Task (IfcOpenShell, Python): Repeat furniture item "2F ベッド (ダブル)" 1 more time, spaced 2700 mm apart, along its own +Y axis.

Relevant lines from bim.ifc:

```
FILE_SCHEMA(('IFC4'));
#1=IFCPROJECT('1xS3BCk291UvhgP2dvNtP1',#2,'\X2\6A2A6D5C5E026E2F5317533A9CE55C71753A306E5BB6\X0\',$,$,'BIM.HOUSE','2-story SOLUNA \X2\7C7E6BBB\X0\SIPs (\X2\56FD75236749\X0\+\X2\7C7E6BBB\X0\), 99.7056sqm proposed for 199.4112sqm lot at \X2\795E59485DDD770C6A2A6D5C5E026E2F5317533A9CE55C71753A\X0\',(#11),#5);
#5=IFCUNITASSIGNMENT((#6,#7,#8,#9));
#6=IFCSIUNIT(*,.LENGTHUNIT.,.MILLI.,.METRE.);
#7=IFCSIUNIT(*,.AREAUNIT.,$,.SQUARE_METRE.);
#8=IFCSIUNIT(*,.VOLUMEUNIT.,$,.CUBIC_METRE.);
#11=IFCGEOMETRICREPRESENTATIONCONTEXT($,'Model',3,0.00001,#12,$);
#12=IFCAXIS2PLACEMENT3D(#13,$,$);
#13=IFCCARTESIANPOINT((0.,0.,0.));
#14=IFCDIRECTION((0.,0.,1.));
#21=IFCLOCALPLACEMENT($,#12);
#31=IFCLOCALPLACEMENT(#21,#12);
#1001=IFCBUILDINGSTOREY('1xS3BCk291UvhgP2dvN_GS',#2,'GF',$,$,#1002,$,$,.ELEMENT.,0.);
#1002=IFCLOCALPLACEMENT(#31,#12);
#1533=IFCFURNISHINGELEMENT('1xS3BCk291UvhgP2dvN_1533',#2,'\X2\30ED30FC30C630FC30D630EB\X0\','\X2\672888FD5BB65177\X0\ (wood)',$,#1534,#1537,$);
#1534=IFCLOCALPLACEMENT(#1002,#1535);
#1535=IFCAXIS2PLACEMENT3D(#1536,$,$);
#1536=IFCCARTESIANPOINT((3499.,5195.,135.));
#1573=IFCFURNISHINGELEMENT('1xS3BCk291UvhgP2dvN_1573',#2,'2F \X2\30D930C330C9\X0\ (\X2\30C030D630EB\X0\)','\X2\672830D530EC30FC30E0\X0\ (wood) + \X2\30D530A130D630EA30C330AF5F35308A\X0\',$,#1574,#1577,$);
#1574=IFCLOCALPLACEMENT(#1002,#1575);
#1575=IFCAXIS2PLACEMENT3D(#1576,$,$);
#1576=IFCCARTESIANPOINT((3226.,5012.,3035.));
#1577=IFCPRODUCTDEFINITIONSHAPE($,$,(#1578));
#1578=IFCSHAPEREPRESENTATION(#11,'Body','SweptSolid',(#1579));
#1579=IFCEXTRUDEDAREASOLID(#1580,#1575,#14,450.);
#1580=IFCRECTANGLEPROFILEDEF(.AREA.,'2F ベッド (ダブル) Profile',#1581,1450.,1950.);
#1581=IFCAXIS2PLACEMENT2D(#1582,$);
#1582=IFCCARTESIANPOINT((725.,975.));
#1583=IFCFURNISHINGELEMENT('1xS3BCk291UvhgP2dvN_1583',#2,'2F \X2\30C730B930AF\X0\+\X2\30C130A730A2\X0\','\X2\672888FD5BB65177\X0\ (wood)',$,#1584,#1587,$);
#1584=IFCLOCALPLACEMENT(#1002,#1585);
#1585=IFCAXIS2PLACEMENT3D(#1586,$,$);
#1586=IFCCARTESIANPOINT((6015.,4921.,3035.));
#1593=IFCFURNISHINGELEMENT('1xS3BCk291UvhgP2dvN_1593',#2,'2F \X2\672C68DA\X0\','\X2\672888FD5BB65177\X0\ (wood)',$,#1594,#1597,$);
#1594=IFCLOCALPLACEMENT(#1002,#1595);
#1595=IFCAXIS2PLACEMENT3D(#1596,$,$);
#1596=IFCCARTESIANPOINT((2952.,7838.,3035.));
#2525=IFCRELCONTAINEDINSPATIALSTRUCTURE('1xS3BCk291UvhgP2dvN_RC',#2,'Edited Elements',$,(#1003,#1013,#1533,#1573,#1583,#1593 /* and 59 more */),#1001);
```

```python
import ifcopenshell
import ifcopenshell.api.geometry
import ifcopenshell.api.root
import ifcopenshell.util.element
import ifcopenshell.util.placement

model = ifcopenshell.open("bim.ifc")


def reuse_history(source, copy):
    """copy_class also copies each property set's owner history, people and application; keep the originals."""
    for rel in copy.IsDefinedBy:
        if rel.is_a("IfcRelDefinesByProperties") and (history := rel.RelatingPropertyDefinition.OwnerHistory):
            rel.RelatingPropertyDefinition.OwnerHistory = source.OwnerHistory
            ifcopenshell.util.element.remove_deep2(model, history)


source = model.by_guid("1xS3BCk291UvhgP2dvN_1573")
base = ifcopenshell.util.placement.get_local_placement(source.ObjectPlacement)
step = base[:3, 1] * 2700.0

for i in range(1, 2):
    copy = ifcopenshell.api.root.copy_class(model, product=source)
    copy.Representation = ifcopenshell.util.element.copy_deep(
        model, source.Representation, exclude=["IfcGeometricRepresentationContext", "IfcRepresentationMap"]
    )
    reuse_history(source, copy)
    matrix = base.copy()
    matrix[:3, 3] += i * step
    print("added at", matrix[:3, 3].round(3) + 0.0)
    ifcopenshell.api.geometry.edit_object_placement(model, product=copy, matrix=matrix, is_si=False)

model.write("bim_updated.ifc")
```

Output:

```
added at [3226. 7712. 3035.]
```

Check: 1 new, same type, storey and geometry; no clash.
